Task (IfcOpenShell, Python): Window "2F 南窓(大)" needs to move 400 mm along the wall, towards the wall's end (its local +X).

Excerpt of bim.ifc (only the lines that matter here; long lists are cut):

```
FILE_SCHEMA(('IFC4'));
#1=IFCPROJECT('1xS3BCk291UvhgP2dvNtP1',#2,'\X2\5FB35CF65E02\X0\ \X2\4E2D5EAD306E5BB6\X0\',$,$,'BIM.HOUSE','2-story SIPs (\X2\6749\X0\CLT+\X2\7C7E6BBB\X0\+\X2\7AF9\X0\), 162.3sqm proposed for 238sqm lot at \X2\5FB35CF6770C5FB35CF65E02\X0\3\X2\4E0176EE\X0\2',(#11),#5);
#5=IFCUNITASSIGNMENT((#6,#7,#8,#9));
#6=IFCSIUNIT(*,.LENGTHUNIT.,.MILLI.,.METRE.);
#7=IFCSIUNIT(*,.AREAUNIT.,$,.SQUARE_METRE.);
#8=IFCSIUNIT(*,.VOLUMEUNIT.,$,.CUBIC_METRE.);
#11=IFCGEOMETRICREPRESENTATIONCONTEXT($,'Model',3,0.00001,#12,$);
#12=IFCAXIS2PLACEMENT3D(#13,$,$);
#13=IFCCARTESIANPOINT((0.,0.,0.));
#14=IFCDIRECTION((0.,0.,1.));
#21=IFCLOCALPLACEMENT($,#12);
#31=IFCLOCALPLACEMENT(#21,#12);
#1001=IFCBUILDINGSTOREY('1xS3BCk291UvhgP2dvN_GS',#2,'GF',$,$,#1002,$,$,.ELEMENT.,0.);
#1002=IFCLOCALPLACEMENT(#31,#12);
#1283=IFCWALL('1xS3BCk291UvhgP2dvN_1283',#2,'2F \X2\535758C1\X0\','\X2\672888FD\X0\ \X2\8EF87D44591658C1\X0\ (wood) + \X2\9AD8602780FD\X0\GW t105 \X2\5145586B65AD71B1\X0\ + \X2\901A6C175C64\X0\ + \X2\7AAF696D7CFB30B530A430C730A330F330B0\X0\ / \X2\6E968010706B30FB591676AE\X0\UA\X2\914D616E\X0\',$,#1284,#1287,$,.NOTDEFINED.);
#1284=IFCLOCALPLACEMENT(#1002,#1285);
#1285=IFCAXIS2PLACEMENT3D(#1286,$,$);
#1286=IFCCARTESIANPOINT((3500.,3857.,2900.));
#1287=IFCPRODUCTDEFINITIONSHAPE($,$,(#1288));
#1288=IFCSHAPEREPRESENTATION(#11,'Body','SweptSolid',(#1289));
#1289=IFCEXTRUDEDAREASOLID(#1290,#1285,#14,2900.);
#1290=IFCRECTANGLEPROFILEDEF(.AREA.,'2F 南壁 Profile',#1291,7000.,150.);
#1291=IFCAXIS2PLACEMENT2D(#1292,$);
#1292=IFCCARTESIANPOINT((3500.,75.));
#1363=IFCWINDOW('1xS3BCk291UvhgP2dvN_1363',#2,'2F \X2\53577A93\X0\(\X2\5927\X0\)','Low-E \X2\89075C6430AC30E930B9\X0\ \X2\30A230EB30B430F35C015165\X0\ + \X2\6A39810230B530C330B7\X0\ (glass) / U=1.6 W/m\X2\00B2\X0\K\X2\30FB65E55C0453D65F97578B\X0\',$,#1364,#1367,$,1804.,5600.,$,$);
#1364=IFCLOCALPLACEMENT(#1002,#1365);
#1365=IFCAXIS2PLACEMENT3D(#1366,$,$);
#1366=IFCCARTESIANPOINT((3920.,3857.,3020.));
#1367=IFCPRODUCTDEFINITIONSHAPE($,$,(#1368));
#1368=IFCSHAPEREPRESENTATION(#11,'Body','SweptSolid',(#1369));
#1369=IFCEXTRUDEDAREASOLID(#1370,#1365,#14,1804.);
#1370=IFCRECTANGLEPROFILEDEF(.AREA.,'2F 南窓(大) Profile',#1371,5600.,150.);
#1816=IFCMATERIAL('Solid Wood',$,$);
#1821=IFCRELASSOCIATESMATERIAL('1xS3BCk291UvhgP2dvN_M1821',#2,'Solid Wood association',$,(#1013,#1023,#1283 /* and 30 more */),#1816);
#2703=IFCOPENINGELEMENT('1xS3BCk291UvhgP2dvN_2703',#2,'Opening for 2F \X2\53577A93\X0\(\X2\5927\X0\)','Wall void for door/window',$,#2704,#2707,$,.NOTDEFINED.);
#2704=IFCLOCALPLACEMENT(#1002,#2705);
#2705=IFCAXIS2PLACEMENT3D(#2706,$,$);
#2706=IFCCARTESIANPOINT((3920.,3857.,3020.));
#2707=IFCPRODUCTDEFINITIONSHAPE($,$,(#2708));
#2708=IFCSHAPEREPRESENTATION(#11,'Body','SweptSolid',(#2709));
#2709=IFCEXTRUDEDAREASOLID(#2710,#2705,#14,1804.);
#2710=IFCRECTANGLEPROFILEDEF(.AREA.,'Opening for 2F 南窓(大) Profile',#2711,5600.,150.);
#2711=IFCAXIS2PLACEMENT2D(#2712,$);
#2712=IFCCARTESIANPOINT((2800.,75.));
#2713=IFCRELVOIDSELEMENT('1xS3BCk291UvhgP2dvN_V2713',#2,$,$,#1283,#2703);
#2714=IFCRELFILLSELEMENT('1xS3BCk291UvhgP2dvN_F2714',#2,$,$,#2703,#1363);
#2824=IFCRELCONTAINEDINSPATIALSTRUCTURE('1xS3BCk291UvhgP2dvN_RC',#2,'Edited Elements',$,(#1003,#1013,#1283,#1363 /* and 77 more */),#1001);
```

```python
import ifcopenshell
import ifcopenshell.api.geometry
import ifcopenshell.util.placement

model = ifcopenshell.open("bim.ifc")

window = model.by_id(1363)
opening = window.FillsVoids[0].RelatingOpeningElement
wall = opening.VoidsElements[0].RelatingBuildingElement

wall_matrix = ifcopenshell.util.placement.get_local_placement(wall.ObjectPlacement)
shift = wall_matrix[:3, 0] * 400.0
before = ifcopenshell.util.placement.get_local_placement(window.ObjectPlacement)[:3, 3].copy()

# The window is not placed relative to its opening, so move both.
for product in (opening, window):
    matrix = ifcopenshell.util.placement.get_local_placement(product.ObjectPlacement)
    matrix[:3, 3] += shift
    ifcopenshell.api.geometry.edit_object_placement(model, product=product, matrix=matrix, is_si=False)

after = ifcopenshell.util.placement.get_local_placement(window.ObjectPlacement)[:3, 3]
print("window moved by", (after - before).round(3) + 0.0)

model.write("bim_updated.ifc")
```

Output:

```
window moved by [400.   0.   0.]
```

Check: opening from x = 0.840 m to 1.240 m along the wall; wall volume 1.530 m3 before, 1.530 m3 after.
